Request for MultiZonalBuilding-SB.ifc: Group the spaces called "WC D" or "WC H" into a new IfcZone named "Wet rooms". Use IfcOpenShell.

First a look at what the model holds.

```python
import ifcopenshell

model = ifcopenshell.open("MultiZonalBuilding-SB.ifc")
print(model.schema)
seen = {}
for space in model.by_type("IfcSpace"):
    seen[space.LongName] = seen.get(space.LongName, 0) + 1
for name, count in sorted(seen.items(), key=str):
    print(count, "x", name)
print("zones:", [z.Name for z in model.by_type("IfcZone")][:20])
```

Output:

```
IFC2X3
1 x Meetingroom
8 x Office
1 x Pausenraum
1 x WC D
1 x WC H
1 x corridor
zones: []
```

```python
import ifcopenshell
import ifcopenshell.api.group
import ifcopenshell.api.root

model = ifcopenshell.open("MultiZonalBuilding-SB.ifc")

names = {"WC D", "WC H"}
spaces = [s for s in model.by_type("IfcSpace") if s.LongName in names]

zone = ifcopenshell.api.root.create_entity(model, ifc_class="IfcZone", name="Wet rooms")
ifcopenshell.api.group.assign_group(model, products=spaces, group=zone)
print(len(spaces), "spaces in", zone.Name)

model.write("MultiZonalBuilding-SB_rev.ifc")
```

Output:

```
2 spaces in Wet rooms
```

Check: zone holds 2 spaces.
